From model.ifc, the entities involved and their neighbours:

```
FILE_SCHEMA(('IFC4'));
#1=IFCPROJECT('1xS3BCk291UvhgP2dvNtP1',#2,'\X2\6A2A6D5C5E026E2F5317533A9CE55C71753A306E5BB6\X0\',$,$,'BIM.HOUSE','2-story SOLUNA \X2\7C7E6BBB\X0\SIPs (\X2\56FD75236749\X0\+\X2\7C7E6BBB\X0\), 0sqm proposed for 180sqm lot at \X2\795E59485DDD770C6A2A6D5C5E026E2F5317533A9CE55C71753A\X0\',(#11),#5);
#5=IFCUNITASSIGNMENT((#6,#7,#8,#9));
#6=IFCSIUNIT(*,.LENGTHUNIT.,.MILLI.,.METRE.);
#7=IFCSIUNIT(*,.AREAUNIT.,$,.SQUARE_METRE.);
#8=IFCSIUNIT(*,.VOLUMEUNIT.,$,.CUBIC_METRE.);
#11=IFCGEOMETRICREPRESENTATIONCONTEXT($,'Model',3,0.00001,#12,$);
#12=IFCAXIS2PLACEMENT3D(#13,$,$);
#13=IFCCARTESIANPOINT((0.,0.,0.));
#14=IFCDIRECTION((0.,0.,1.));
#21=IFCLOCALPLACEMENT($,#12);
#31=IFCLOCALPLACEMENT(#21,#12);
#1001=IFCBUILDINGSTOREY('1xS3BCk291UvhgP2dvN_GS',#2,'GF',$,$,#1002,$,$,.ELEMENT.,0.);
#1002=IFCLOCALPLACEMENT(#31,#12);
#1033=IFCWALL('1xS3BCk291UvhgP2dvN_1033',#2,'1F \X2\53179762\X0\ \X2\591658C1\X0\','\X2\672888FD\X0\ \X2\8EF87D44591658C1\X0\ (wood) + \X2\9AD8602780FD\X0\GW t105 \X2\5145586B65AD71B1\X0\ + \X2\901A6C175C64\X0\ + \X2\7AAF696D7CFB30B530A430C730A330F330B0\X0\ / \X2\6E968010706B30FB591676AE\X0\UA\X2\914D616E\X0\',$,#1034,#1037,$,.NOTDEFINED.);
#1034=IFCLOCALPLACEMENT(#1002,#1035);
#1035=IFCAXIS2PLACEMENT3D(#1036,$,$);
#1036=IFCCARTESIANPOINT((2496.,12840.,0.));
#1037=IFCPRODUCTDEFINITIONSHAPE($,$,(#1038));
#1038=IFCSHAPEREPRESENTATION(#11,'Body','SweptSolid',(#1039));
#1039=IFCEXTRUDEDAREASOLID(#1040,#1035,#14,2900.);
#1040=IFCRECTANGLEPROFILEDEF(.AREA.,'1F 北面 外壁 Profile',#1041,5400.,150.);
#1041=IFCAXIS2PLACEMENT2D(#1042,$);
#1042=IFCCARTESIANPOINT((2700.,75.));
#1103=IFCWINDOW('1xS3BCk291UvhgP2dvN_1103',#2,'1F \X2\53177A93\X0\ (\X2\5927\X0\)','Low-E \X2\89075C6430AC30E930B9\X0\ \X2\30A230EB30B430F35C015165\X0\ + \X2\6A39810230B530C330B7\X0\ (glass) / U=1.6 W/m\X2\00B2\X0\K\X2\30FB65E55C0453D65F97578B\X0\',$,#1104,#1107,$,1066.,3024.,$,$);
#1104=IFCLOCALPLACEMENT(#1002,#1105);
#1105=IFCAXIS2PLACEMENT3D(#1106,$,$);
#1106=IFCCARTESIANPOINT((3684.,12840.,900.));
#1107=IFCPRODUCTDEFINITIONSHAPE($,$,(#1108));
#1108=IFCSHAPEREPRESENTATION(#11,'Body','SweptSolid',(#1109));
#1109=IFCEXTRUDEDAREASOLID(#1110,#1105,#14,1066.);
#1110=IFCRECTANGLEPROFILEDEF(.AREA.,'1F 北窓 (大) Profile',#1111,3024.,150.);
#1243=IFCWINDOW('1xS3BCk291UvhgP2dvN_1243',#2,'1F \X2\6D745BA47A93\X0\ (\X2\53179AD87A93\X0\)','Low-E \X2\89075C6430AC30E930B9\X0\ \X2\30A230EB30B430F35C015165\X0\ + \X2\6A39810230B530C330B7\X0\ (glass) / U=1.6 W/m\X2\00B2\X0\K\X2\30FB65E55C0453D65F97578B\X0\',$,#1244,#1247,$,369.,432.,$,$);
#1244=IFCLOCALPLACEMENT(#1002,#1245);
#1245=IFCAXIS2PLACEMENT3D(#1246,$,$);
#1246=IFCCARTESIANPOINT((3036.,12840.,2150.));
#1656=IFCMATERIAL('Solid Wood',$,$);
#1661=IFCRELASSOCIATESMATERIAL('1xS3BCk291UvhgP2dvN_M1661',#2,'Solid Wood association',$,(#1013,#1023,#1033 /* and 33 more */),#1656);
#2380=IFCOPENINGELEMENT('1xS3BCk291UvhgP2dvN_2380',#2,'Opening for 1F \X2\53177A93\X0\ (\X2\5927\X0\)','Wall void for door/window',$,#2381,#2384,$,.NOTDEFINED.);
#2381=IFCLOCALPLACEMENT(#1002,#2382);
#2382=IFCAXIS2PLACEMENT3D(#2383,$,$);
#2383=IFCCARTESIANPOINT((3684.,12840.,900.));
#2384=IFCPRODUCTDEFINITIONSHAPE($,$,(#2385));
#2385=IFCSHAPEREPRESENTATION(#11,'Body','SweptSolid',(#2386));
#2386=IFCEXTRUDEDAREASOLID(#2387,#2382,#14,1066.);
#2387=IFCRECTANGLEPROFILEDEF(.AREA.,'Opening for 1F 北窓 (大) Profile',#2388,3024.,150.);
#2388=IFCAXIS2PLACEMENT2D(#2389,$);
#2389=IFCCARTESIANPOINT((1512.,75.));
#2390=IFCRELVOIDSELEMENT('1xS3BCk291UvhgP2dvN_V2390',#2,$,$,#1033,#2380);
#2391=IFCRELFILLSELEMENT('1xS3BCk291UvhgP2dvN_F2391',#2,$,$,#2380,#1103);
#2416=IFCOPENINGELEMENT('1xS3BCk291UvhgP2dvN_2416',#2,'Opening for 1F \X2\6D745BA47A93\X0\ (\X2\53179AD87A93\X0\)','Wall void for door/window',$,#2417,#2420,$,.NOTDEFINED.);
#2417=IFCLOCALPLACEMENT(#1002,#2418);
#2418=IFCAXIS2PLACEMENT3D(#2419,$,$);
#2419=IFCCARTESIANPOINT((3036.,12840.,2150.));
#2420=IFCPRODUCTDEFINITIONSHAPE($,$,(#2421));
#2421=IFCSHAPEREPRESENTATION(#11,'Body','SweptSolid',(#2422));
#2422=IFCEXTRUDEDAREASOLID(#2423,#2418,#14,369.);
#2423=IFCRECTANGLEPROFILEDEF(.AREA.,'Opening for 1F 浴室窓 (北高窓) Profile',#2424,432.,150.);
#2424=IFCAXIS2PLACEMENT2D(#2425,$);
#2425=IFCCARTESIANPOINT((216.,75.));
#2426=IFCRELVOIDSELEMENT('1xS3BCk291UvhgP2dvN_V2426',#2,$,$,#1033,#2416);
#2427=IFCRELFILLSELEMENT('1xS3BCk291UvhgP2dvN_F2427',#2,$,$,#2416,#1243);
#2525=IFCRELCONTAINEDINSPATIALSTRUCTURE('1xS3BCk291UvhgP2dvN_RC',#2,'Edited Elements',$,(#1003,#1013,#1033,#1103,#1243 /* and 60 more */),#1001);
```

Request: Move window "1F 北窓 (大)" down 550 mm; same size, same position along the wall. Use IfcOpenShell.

```python
import numpy as np
import ifcopenshell
import ifcopenshell.api.geometry
import ifcopenshell.util.placement
import ifcopenshell.util.unit

model = ifcopenshell.open("model.ifc")
unit_scale = ifcopenshell.util.unit.calculate_unit_scale(model)

window = model.by_id(1103)
opening = window.FillsVoids[0].RelatingOpeningElement
dz = -0.55 / unit_scale

shift = np.array([0.0, 0.0, dz])
# The window is not placed relative to its opening, so move both.
for product in (opening, window):
    matrix = ifcopenshell.util.placement.get_local_placement(product.ObjectPlacement)
    matrix[:3, 3] += shift
    ifcopenshell.api.geometry.edit_object_placement(model, product=product, matrix=matrix, is_si=False)

print(f"moved by {dz * unit_scale:+.3f} m")

model.write("model_edited.ifc")
```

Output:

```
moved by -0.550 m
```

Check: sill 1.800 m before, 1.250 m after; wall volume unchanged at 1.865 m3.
